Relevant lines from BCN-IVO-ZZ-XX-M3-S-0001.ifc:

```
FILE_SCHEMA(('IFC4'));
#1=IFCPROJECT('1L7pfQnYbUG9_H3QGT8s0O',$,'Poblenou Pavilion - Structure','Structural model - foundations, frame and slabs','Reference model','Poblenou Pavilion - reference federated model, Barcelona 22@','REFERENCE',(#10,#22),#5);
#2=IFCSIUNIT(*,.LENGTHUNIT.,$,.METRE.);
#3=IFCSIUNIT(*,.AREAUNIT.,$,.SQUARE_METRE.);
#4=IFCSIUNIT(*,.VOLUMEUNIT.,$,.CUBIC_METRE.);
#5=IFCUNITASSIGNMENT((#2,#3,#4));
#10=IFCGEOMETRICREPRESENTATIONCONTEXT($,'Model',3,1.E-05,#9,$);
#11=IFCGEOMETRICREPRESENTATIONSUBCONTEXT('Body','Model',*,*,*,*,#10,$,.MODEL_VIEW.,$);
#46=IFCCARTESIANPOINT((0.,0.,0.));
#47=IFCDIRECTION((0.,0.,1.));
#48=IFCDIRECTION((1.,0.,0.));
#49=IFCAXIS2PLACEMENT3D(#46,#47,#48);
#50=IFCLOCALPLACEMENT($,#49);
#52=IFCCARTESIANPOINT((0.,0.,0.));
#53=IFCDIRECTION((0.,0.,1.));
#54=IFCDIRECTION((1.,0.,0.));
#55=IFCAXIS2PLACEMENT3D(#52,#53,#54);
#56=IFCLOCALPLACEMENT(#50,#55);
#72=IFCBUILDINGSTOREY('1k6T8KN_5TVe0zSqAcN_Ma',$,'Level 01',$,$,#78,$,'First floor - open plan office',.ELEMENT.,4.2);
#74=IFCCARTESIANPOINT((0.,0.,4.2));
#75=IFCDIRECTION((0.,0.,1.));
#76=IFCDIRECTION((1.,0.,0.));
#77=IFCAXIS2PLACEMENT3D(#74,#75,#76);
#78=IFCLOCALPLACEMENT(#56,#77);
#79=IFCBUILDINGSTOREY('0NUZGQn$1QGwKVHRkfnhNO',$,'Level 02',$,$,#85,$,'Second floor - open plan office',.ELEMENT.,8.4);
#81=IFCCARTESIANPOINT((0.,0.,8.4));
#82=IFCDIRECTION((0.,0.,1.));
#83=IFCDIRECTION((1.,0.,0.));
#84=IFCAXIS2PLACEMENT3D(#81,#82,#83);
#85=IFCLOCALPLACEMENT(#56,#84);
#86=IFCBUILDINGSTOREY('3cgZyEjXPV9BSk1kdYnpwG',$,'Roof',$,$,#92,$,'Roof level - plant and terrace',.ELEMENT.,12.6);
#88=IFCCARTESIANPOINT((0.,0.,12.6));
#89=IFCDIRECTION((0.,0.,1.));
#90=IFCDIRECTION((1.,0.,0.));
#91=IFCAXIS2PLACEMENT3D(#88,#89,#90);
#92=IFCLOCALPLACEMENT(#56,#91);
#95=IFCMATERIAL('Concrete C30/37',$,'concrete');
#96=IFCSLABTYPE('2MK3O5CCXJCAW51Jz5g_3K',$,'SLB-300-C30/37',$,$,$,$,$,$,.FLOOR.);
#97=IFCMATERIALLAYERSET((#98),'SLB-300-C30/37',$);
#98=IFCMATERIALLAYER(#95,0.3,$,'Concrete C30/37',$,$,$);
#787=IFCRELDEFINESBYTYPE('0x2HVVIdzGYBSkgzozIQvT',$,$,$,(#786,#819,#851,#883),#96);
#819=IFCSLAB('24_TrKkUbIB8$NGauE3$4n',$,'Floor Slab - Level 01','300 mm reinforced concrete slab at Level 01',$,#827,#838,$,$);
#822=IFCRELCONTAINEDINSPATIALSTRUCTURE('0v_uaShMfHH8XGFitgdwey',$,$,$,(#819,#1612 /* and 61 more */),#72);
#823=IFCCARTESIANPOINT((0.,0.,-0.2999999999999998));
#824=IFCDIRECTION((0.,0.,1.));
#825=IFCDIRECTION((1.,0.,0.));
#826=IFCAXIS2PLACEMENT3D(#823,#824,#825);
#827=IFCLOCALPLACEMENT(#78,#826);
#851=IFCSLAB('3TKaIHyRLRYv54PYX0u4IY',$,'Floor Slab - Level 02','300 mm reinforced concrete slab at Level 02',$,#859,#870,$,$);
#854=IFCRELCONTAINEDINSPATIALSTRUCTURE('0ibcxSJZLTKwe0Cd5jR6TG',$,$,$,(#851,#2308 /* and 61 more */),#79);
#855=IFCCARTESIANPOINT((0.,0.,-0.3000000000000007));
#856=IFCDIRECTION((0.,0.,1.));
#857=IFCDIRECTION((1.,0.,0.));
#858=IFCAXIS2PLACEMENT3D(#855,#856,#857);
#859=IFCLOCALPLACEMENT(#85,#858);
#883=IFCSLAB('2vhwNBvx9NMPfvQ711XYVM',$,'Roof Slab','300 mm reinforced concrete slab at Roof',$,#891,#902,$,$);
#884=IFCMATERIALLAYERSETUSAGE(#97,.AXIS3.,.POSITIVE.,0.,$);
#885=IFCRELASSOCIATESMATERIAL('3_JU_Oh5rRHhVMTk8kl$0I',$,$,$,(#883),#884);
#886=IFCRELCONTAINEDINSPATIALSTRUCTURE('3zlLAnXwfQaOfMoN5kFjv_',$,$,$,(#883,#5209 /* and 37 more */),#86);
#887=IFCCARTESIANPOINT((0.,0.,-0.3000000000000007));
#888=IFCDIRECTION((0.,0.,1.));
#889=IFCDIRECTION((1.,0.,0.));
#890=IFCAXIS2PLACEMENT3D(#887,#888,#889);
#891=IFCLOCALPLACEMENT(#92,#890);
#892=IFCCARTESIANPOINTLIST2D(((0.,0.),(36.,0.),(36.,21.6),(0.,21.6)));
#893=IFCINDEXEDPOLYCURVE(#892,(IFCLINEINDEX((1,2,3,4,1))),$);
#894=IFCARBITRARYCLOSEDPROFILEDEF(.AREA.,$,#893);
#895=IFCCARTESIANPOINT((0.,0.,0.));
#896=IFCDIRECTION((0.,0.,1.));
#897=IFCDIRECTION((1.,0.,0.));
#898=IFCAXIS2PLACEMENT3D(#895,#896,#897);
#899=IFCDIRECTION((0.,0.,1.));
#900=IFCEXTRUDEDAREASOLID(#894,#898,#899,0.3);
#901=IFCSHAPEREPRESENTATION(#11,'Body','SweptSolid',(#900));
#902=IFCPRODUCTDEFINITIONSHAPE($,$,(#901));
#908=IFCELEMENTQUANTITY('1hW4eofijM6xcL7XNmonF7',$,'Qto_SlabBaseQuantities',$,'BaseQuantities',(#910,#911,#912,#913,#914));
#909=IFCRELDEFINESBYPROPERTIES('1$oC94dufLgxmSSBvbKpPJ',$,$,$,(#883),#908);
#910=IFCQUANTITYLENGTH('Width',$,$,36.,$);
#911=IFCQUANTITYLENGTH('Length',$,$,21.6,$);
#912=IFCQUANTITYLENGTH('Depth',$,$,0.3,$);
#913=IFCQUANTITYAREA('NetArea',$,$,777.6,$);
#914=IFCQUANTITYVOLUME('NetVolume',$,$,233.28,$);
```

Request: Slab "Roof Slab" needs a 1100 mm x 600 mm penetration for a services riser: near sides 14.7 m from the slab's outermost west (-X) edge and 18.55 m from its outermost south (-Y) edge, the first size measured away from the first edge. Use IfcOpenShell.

```python
import numpy as np
import ifcopenshell
import ifcopenshell.api.feature
import ifcopenshell.api.geometry
import ifcopenshell.api.pset
import ifcopenshell.api.root
import ifcopenshell.geom
import ifcopenshell.util.element
import ifcopenshell.util.placement
import ifcopenshell.util.representation
import ifcopenshell.util.shape
import ifcopenshell.util.unit

model = ifcopenshell.open("BCN-IVO-ZZ-XX-M3-S-0001.ifc")
unit_scale = ifcopenshell.util.unit.calculate_unit_scale(model)
area_scale = ifcopenshell.util.unit.calculate_unit_scale(model, "AREAUNIT")
volume_scale = ifcopenshell.util.unit.calculate_unit_scale(model, "VOLUMEUNIT")
settings = ifcopenshell.geom.settings()


def volume(element):
    """Net volume in cubic metres, openings subtracted."""
    shape = ifcopenshell.geom.create_shape(settings, element)
    return ifcopenshell.util.shape.get_volume(shape.geometry)


slab = model.by_guid("2vhwNBvx9NMPfvQ711XYVM")
before = volume(slab)

# Extent in the slab's own axes, in metres. The edges named are its -X and -Y sides.
slab_shape = ifcopenshell.geom.create_shape(settings, slab)
vertices = ifcopenshell.util.shape.get_vertices(slab_shape.geometry)
x_min, y_min, bottom = vertices.min(axis=0)
top = vertices[:, 2].max()

opening = ifcopenshell.api.root.create_entity(model, ifc_class="IfcOpeningElement", name="Services riser opening", predefined_type="OPENING")
context = ifcopenshell.util.representation.get_context(model, "Model", "Body", "MODEL_VIEW")
width, depth = 1.1, 0.6
outline = [(0.0, 0.0), (width, 0.0), (width, depth), (0.0, depth), (0.0, 0.0)]
# Overshoot both faces by 50 mm so the cut is clean.
shape = ifcopenshell.api.geometry.add_slab_representation(
    model, context=context, depth=top - bottom + 0.1, polyline=outline
)
ifcopenshell.api.geometry.assign_representation(model, product=opening, representation=shape)

matrix = ifcopenshell.util.placement.get_local_placement(slab.ObjectPlacement)
matrix[:, 3] = matrix @ np.append(np.array([x_min + 14.7, y_min + 18.55, bottom - 0.05]) / unit_scale, 1.0)
ifcopenshell.api.geometry.edit_object_placement(model, product=opening, matrix=matrix, is_si=False)
ifcopenshell.api.feature.add_feature(model, feature=opening, element=slab)

after = volume(slab)

# Update the slab's stored quantities.
qto = model.by_id(ifcopenshell.util.element.get_pset(slab, "Qto_SlabBaseQuantities", should_inherit=False)["id"])
ifcopenshell.api.pset.edit_qto(model, qto=qto, properties={
    "NetArea": after / (top - bottom) / area_scale,
    "NetVolume": after / volume_scale,
})

print(f"slab volume {before:.3f} -> {after:.3f} m3")

model.write("BCN-IVO-ZZ-XX-M3-S-0001_updated.ifc")
```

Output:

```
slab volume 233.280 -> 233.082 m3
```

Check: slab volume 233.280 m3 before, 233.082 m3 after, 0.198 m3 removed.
